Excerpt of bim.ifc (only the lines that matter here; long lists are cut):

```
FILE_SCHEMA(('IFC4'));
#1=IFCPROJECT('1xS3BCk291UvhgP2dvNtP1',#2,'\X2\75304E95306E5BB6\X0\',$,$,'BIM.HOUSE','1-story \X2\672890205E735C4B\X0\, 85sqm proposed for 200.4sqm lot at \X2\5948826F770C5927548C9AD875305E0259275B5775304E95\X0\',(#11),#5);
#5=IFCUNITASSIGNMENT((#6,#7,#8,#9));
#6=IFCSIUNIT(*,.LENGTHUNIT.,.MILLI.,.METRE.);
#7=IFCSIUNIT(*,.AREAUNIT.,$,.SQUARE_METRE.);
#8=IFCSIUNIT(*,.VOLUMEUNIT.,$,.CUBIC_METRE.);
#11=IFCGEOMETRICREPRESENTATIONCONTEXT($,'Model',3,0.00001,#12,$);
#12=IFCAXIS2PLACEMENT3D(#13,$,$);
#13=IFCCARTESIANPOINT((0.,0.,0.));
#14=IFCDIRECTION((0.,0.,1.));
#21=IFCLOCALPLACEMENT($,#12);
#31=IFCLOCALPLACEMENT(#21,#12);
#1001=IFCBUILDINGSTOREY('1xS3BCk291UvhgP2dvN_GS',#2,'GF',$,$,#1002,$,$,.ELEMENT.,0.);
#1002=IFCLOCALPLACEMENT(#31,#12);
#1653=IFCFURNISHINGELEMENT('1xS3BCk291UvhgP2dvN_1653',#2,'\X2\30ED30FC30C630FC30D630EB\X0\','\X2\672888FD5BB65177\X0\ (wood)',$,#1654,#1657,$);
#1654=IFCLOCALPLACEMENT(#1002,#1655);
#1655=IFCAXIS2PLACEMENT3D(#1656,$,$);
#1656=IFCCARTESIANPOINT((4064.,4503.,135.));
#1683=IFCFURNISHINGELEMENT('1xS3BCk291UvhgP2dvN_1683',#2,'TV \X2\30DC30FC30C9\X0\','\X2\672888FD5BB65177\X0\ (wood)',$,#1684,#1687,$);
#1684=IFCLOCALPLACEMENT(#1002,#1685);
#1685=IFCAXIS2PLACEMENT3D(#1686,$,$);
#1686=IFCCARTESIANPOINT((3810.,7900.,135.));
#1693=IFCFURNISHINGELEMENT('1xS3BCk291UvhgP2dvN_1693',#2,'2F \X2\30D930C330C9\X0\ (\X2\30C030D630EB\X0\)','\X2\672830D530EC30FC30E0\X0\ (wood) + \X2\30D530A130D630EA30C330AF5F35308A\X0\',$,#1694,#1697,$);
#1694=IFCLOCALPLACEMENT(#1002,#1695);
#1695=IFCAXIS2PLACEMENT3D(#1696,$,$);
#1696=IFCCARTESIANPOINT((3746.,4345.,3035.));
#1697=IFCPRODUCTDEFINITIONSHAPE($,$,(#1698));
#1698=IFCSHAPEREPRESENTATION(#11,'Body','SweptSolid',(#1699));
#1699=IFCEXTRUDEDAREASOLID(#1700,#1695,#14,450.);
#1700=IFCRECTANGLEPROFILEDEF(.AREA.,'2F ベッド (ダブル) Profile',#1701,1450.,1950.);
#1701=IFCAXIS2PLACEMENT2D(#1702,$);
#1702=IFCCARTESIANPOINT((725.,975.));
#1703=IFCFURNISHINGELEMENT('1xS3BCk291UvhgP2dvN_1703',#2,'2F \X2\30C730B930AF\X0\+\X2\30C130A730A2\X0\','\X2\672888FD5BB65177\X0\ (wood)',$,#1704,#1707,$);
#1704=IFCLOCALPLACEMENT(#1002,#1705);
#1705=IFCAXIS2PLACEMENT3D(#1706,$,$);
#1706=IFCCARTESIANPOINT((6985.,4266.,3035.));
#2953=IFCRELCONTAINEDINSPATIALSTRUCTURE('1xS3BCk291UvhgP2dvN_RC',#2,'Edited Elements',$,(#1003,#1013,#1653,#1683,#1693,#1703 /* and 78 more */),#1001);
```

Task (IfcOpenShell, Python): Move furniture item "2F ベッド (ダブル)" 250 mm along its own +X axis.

```python
import ifcopenshell
import ifcopenshell.api.geometry
import ifcopenshell.util.placement

model = ifcopenshell.open("bim.ifc")

item = model.by_guid("1xS3BCk291UvhgP2dvN_1693")
matrix = ifcopenshell.util.placement.get_local_placement(item.ObjectPlacement)
matrix[:3, 3] += matrix[:3, 0] * 250.0
ifcopenshell.api.geometry.edit_object_placement(model, product=item, matrix=matrix, is_si=False)

print(ifcopenshell.util.placement.get_local_placement(item.ObjectPlacement).round(3) + 0.0)

model.write("bim-out.ifc")
```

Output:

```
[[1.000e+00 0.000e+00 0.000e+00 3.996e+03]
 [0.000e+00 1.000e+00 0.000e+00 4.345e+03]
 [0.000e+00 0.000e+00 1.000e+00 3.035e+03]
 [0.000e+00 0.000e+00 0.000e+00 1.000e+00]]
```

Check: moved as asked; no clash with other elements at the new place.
